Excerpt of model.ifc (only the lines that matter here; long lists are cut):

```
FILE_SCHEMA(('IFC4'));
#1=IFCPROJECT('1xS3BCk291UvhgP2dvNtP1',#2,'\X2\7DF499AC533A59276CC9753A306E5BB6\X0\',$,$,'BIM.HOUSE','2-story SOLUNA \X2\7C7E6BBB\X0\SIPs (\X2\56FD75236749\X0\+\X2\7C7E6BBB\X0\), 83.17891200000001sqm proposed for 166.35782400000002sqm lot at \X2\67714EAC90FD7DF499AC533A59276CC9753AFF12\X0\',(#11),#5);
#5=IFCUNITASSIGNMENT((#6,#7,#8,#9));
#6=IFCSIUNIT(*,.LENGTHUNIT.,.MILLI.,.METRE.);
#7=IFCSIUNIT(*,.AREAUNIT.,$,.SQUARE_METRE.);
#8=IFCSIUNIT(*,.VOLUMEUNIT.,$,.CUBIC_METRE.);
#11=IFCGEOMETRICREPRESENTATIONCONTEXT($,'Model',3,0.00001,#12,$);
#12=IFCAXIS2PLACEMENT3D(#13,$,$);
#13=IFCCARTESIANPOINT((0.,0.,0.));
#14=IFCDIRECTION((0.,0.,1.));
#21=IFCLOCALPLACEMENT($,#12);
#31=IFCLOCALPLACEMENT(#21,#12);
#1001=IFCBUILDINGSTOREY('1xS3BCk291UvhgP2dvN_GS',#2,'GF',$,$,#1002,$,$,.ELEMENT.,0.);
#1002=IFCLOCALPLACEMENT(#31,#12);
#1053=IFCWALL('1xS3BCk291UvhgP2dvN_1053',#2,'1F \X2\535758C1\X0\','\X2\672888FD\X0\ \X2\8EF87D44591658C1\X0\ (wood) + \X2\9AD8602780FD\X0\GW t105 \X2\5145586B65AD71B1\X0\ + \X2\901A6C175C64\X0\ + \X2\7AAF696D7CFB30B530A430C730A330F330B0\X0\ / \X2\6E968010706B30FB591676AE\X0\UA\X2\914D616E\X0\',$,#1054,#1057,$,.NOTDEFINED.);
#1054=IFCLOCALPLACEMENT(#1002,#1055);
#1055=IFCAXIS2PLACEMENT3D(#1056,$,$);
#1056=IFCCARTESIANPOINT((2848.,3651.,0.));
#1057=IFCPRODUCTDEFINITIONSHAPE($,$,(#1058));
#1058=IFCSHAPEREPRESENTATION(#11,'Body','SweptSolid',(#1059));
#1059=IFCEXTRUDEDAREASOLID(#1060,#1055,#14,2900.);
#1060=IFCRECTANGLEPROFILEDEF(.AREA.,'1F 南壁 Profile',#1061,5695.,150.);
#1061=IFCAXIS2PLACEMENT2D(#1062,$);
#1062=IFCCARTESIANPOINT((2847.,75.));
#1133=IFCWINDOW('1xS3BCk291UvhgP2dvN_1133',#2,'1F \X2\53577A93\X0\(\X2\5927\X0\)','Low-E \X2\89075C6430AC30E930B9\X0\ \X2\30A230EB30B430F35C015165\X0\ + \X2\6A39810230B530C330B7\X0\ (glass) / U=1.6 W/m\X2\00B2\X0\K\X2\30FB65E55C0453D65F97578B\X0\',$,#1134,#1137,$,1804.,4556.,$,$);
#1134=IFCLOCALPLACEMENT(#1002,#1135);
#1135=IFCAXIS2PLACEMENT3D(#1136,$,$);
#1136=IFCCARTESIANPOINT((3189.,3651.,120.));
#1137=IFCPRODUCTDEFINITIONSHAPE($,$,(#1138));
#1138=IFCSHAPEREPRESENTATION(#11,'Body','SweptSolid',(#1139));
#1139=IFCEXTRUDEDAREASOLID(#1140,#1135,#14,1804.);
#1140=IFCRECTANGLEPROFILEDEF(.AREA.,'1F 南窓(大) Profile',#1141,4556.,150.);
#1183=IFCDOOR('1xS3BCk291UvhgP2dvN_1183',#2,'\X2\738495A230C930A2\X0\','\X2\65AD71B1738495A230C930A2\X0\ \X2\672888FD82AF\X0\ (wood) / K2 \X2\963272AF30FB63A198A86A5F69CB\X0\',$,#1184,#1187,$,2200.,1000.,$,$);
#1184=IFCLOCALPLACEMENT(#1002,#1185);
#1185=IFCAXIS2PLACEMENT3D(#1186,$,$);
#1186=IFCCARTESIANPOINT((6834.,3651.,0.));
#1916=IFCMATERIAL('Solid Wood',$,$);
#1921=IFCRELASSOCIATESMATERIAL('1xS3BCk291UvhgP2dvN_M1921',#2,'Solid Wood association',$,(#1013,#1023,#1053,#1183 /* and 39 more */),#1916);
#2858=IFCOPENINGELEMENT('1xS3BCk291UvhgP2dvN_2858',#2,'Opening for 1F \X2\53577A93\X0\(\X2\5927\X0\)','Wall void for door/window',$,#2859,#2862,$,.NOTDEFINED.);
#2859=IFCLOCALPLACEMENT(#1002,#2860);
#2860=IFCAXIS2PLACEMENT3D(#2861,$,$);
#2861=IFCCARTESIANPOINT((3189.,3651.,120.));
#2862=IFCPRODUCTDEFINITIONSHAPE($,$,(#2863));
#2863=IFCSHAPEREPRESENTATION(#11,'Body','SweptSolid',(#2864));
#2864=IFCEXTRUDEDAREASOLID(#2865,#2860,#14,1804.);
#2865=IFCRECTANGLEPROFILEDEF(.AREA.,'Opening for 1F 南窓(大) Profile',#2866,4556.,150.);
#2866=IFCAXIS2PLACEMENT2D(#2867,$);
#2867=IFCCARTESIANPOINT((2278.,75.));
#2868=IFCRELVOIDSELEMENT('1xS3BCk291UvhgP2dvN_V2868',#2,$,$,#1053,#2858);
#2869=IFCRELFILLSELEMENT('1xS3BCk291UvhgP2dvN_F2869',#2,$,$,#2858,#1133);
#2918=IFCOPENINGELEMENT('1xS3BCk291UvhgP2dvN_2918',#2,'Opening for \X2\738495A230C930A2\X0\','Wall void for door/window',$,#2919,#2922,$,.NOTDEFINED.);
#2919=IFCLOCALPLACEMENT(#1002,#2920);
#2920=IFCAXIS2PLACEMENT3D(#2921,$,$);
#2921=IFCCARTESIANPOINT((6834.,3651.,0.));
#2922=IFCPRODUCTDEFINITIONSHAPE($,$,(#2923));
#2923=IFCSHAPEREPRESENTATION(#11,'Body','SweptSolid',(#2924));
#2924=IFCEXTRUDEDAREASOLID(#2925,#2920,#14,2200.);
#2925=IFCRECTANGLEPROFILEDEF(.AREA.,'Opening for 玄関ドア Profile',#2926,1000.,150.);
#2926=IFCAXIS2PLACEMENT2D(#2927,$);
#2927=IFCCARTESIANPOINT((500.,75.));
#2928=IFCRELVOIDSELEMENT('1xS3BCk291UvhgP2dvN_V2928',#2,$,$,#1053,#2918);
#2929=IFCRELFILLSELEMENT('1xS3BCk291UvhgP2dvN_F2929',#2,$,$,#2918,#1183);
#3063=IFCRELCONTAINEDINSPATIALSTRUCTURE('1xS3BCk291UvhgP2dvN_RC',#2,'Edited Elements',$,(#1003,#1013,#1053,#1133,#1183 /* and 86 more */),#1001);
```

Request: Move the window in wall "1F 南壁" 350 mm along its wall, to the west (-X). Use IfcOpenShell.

```python
import ifcopenshell
import ifcopenshell.api.geometry
import ifcopenshell.util.placement
import ifcopenshell.util.unit

model = ifcopenshell.open("model.ifc")
unit_scale = ifcopenshell.util.unit.calculate_unit_scale(model)

window = model.by_guid("1xS3BCk291UvhgP2dvN_1133")
opening = window.FillsVoids[0].RelatingOpeningElement
wall = opening.VoidsElements[0].RelatingBuildingElement

wall_matrix = ifcopenshell.util.placement.get_local_placement(wall.ObjectPlacement)
shift = wall_matrix[:3, 0] * -0.35 / unit_scale
before = ifcopenshell.util.placement.get_local_placement(window.ObjectPlacement)[:3, 3].copy()

# The window is not placed relative to its opening, so move both.
for product in (opening, window):
    matrix = ifcopenshell.util.placement.get_local_placement(product.ObjectPlacement)
    matrix[:3, 3] += shift
    ifcopenshell.api.geometry.edit_object_placement(model, product=product, matrix=matrix, is_si=False)

after = ifcopenshell.util.placement.get_local_placement(window.ObjectPlacement)[:3, 3]
print("window moved by", (after - before).round(3) + 0.0)

model.write("model_updated.ifc")
```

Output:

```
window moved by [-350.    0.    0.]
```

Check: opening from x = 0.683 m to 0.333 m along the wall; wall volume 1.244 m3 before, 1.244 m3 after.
